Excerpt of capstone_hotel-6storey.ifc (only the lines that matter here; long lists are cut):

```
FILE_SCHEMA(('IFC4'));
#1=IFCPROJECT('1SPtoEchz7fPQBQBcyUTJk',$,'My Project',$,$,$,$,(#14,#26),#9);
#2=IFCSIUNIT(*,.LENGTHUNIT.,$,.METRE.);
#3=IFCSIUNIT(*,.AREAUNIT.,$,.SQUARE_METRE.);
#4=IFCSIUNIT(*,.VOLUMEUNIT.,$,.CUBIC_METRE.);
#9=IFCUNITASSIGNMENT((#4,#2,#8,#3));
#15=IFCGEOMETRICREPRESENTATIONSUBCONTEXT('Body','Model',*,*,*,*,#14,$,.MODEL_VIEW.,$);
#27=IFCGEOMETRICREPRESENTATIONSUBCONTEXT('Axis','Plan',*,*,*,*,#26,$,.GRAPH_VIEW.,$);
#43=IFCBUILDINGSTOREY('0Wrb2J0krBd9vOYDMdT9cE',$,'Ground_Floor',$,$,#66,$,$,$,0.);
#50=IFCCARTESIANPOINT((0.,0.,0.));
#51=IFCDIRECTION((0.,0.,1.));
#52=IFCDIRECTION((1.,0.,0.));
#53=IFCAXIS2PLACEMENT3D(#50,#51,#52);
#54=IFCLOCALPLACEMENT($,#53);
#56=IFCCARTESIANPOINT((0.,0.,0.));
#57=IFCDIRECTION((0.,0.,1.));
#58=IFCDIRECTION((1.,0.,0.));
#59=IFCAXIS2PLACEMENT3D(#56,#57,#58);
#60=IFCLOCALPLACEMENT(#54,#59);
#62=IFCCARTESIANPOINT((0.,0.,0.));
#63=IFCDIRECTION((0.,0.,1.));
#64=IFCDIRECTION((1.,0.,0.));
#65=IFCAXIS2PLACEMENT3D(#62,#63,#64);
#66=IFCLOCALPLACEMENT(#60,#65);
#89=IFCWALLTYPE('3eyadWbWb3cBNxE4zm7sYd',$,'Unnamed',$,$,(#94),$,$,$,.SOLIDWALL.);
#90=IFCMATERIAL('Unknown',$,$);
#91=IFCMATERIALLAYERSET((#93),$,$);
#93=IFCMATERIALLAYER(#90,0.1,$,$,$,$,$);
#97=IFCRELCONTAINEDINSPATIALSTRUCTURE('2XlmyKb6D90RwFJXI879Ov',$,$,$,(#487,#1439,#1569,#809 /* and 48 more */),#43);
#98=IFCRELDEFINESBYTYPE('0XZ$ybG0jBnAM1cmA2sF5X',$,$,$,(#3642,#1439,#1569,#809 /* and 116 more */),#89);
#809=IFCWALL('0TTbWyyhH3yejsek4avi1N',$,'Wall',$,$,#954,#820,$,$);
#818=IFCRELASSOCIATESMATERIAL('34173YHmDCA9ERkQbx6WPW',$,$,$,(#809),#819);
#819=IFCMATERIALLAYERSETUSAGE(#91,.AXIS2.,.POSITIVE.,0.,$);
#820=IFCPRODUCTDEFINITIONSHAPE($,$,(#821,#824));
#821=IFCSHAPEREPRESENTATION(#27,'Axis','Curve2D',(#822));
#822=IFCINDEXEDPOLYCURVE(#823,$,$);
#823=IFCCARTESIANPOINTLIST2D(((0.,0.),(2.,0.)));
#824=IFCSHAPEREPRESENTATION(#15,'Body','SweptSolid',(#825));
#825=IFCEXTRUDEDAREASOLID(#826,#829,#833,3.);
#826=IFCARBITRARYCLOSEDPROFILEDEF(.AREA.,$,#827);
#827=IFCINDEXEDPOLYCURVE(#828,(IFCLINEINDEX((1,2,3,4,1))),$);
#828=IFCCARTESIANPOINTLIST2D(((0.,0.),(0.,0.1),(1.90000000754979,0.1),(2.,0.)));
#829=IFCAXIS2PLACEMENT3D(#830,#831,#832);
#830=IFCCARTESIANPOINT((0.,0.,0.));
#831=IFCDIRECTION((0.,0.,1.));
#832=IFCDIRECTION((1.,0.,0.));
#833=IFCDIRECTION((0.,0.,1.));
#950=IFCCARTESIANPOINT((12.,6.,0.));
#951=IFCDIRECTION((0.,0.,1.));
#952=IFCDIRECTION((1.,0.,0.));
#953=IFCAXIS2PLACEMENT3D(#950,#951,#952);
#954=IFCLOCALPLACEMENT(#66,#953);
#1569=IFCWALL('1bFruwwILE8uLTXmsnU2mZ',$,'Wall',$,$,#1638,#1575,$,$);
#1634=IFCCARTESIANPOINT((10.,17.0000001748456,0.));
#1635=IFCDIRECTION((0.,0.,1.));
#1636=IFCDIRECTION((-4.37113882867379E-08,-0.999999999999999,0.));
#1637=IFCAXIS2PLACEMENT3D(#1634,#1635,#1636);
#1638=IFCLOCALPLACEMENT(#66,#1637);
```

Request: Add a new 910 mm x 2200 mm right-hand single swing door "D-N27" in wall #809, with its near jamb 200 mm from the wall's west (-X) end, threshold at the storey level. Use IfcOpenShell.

```python
import numpy as np
import ifcopenshell
import ifcopenshell.api.feature
import ifcopenshell.api.geometry
import ifcopenshell.api.root
import ifcopenshell.api.spatial
import ifcopenshell.geom
import ifcopenshell.util.element
import ifcopenshell.util.placement
import ifcopenshell.util.representation
import ifcopenshell.util.shape
import ifcopenshell.util.unit

model = ifcopenshell.open("capstone_hotel-6storey.ifc")
unit_scale = ifcopenshell.util.unit.calculate_unit_scale(model)
settings = ifcopenshell.geom.settings()


def volume(element):
    """Net volume in cubic metres, openings subtracted."""
    shape = ifcopenshell.geom.create_shape(settings, element)
    return ifcopenshell.util.shape.get_volume(shape.geometry)


wall = model.by_guid("0TTbWyyhH3yejsek4avi1N")
storey = ifcopenshell.util.element.get_container(wall, ifc_class="IfcBuildingStorey")
context = ifcopenshell.util.representation.get_context(model, "Model", "Body", "MODEL_VIEW")
before = volume(wall)

width, height, from_end, sill = 0.91, 2.2, 0.2, 0.0  # metres

# The wall runs along its own X axis, and the end named is its -X end.
wall_shape = ifcopenshell.geom.create_shape(settings, wall)
x, y, z = ifcopenshell.util.shape.get_vertices(wall_shape.geometry).T
start = x.min() + from_end
face, thickness = float(y.min()), float(y.max() - y.min())
wall_matrix = ifcopenshell.util.placement.get_local_placement(wall.ObjectPlacement)
level = ifcopenshell.util.placement.get_local_placement(storey.ObjectPlacement)[2, 3]


def in_wall(x, y):
    """Placement at x, y metres in the wall's axes, at sill height."""
    matrix = wall_matrix.copy()
    matrix[:, 3] = wall_matrix @ np.array([x / unit_scale, y / unit_scale, 0.0, 1.0])
    matrix[2, 3] = level + sill / unit_scale
    return matrix


# Opening: a box that overshoots both wall faces by 50 mm.
opening = ifcopenshell.api.root.create_entity(model, ifc_class="IfcOpeningElement", predefined_type="OPENING")
box = ifcopenshell.api.geometry.add_wall_representation(
    model, context=context, length=width, height=height, thickness=thickness + 0.1
)
ifcopenshell.api.geometry.assign_representation(model, product=opening, representation=box)
ifcopenshell.api.geometry.edit_object_placement(model, product=opening, matrix=in_wall(start, face - 0.05), is_si=False)
ifcopenshell.api.feature.add_feature(model, feature=opening, element=wall)

door = ifcopenshell.api.root.create_entity(model, ifc_class="IfcDoor", name="D-N27", predefined_type="DOOR")
door.OverallWidth, door.OverallHeight = width / unit_scale, height / unit_scale
door.OperationType = "SINGLE_SWING_RIGHT"
body = ifcopenshell.api.geometry.add_door_representation(
    model,
    context=context,
    overall_width=door.OverallWidth,
    overall_height=door.OverallHeight,
    operation_type="SINGLE_SWING_RIGHT",
    lining_properties={"LiningDepth": thickness / unit_scale, "ThresholdDepth": thickness / unit_scale},
)
ifcopenshell.api.geometry.assign_representation(model, product=door, representation=body)
ifcopenshell.api.spatial.assign_container(model, products=[door], relating_structure=storey)
ifcopenshell.api.feature.add_filling(model, opening=opening, element=door)

# The lining spans the wall, so the door starts at the wall face.
ifcopenshell.api.geometry.edit_object_placement(model, product=door, matrix=in_wall(start, face), is_si=False)

after = volume(wall)

print(f"wall volume {before:.3f} -> {after:.3f} m3")

model.write("capstone_hotel-6storey-out.ifc")
```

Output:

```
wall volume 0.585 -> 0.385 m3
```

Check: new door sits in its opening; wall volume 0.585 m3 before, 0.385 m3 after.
